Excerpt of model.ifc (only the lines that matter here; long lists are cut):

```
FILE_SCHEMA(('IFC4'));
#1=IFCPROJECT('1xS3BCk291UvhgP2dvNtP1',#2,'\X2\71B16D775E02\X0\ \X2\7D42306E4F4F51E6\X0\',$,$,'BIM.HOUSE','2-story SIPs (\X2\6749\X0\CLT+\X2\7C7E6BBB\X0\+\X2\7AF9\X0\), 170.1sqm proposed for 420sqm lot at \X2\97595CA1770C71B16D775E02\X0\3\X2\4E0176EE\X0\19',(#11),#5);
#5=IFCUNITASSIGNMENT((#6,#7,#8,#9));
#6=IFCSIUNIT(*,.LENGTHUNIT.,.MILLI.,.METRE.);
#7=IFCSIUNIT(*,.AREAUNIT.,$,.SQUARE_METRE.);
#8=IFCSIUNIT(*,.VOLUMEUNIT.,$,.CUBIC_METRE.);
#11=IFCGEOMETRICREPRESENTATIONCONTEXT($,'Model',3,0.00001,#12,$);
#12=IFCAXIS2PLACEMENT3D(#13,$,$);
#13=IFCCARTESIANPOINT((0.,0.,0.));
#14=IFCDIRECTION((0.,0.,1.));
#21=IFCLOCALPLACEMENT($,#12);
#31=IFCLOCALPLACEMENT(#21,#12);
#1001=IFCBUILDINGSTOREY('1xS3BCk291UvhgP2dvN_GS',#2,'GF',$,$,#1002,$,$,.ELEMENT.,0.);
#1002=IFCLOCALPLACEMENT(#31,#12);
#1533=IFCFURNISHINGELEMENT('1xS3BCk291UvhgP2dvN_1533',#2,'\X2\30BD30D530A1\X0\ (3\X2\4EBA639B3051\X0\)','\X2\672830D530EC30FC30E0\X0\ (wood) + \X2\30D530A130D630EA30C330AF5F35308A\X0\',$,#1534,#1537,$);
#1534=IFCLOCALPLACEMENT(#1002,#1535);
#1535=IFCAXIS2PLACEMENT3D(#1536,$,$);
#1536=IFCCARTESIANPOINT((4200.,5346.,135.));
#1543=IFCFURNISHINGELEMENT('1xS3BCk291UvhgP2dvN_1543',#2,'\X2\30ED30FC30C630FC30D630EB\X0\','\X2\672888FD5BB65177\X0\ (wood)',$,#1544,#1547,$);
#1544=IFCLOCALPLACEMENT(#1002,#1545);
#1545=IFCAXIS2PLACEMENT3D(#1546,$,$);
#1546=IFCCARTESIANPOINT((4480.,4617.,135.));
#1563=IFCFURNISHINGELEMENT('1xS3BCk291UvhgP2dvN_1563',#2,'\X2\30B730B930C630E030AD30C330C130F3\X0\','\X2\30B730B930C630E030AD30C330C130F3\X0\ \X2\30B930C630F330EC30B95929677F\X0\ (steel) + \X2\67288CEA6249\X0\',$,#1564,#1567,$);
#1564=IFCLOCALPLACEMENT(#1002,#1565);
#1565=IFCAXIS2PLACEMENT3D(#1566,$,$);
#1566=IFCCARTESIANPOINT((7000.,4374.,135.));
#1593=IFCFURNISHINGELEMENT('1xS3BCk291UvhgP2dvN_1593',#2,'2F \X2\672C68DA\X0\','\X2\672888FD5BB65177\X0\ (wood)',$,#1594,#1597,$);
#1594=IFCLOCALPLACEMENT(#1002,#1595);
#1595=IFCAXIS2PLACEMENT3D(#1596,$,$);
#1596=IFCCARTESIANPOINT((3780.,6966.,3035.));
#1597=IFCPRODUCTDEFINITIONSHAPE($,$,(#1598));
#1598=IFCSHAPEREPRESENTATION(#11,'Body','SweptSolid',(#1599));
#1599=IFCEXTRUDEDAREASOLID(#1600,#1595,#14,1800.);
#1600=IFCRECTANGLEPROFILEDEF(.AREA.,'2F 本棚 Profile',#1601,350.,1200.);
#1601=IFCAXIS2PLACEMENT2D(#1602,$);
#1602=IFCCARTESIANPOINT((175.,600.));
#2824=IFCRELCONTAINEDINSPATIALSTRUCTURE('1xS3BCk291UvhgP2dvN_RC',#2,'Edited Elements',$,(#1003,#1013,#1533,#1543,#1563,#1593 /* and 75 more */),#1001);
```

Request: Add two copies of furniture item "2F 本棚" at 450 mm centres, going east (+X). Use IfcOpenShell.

```python
import numpy as np
import ifcopenshell
import ifcopenshell.api.geometry
import ifcopenshell.api.root
import ifcopenshell.util.element
import ifcopenshell.util.placement

model = ifcopenshell.open("model.ifc")


def reuse_history(source, copy):
    """copy_class also copies each property set's owner history, people and application; keep the originals."""
    for rel in copy.IsDefinedBy:
        if rel.is_a("IfcRelDefinesByProperties") and (history := rel.RelatingPropertyDefinition.OwnerHistory):
            rel.RelatingPropertyDefinition.OwnerHistory = source.OwnerHistory
            ifcopenshell.util.element.remove_deep2(model, history)


source = model.by_guid("1xS3BCk291UvhgP2dvN_1593")
base = ifcopenshell.util.placement.get_local_placement(source.ObjectPlacement)
step = np.array([1.0, 0.0, 0.0]) * 450.0

for i in range(1, 3):
    copy = ifcopenshell.api.root.copy_class(model, product=source)
    copy.Representation = ifcopenshell.util.element.copy_deep(
        model, source.Representation, exclude=["IfcGeometricRepresentationContext", "IfcRepresentationMap"]
    )
    reuse_history(source, copy)
    matrix = base.copy()
    matrix[:3, 3] += i * step
    print("added at", matrix[:3, 3].round(3) + 0.0)
    ifcopenshell.api.geometry.edit_object_placement(model, product=copy, matrix=matrix, is_si=False)

model.write("model_edited.ifc")
```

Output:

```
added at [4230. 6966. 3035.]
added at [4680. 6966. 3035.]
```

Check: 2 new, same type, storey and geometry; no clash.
